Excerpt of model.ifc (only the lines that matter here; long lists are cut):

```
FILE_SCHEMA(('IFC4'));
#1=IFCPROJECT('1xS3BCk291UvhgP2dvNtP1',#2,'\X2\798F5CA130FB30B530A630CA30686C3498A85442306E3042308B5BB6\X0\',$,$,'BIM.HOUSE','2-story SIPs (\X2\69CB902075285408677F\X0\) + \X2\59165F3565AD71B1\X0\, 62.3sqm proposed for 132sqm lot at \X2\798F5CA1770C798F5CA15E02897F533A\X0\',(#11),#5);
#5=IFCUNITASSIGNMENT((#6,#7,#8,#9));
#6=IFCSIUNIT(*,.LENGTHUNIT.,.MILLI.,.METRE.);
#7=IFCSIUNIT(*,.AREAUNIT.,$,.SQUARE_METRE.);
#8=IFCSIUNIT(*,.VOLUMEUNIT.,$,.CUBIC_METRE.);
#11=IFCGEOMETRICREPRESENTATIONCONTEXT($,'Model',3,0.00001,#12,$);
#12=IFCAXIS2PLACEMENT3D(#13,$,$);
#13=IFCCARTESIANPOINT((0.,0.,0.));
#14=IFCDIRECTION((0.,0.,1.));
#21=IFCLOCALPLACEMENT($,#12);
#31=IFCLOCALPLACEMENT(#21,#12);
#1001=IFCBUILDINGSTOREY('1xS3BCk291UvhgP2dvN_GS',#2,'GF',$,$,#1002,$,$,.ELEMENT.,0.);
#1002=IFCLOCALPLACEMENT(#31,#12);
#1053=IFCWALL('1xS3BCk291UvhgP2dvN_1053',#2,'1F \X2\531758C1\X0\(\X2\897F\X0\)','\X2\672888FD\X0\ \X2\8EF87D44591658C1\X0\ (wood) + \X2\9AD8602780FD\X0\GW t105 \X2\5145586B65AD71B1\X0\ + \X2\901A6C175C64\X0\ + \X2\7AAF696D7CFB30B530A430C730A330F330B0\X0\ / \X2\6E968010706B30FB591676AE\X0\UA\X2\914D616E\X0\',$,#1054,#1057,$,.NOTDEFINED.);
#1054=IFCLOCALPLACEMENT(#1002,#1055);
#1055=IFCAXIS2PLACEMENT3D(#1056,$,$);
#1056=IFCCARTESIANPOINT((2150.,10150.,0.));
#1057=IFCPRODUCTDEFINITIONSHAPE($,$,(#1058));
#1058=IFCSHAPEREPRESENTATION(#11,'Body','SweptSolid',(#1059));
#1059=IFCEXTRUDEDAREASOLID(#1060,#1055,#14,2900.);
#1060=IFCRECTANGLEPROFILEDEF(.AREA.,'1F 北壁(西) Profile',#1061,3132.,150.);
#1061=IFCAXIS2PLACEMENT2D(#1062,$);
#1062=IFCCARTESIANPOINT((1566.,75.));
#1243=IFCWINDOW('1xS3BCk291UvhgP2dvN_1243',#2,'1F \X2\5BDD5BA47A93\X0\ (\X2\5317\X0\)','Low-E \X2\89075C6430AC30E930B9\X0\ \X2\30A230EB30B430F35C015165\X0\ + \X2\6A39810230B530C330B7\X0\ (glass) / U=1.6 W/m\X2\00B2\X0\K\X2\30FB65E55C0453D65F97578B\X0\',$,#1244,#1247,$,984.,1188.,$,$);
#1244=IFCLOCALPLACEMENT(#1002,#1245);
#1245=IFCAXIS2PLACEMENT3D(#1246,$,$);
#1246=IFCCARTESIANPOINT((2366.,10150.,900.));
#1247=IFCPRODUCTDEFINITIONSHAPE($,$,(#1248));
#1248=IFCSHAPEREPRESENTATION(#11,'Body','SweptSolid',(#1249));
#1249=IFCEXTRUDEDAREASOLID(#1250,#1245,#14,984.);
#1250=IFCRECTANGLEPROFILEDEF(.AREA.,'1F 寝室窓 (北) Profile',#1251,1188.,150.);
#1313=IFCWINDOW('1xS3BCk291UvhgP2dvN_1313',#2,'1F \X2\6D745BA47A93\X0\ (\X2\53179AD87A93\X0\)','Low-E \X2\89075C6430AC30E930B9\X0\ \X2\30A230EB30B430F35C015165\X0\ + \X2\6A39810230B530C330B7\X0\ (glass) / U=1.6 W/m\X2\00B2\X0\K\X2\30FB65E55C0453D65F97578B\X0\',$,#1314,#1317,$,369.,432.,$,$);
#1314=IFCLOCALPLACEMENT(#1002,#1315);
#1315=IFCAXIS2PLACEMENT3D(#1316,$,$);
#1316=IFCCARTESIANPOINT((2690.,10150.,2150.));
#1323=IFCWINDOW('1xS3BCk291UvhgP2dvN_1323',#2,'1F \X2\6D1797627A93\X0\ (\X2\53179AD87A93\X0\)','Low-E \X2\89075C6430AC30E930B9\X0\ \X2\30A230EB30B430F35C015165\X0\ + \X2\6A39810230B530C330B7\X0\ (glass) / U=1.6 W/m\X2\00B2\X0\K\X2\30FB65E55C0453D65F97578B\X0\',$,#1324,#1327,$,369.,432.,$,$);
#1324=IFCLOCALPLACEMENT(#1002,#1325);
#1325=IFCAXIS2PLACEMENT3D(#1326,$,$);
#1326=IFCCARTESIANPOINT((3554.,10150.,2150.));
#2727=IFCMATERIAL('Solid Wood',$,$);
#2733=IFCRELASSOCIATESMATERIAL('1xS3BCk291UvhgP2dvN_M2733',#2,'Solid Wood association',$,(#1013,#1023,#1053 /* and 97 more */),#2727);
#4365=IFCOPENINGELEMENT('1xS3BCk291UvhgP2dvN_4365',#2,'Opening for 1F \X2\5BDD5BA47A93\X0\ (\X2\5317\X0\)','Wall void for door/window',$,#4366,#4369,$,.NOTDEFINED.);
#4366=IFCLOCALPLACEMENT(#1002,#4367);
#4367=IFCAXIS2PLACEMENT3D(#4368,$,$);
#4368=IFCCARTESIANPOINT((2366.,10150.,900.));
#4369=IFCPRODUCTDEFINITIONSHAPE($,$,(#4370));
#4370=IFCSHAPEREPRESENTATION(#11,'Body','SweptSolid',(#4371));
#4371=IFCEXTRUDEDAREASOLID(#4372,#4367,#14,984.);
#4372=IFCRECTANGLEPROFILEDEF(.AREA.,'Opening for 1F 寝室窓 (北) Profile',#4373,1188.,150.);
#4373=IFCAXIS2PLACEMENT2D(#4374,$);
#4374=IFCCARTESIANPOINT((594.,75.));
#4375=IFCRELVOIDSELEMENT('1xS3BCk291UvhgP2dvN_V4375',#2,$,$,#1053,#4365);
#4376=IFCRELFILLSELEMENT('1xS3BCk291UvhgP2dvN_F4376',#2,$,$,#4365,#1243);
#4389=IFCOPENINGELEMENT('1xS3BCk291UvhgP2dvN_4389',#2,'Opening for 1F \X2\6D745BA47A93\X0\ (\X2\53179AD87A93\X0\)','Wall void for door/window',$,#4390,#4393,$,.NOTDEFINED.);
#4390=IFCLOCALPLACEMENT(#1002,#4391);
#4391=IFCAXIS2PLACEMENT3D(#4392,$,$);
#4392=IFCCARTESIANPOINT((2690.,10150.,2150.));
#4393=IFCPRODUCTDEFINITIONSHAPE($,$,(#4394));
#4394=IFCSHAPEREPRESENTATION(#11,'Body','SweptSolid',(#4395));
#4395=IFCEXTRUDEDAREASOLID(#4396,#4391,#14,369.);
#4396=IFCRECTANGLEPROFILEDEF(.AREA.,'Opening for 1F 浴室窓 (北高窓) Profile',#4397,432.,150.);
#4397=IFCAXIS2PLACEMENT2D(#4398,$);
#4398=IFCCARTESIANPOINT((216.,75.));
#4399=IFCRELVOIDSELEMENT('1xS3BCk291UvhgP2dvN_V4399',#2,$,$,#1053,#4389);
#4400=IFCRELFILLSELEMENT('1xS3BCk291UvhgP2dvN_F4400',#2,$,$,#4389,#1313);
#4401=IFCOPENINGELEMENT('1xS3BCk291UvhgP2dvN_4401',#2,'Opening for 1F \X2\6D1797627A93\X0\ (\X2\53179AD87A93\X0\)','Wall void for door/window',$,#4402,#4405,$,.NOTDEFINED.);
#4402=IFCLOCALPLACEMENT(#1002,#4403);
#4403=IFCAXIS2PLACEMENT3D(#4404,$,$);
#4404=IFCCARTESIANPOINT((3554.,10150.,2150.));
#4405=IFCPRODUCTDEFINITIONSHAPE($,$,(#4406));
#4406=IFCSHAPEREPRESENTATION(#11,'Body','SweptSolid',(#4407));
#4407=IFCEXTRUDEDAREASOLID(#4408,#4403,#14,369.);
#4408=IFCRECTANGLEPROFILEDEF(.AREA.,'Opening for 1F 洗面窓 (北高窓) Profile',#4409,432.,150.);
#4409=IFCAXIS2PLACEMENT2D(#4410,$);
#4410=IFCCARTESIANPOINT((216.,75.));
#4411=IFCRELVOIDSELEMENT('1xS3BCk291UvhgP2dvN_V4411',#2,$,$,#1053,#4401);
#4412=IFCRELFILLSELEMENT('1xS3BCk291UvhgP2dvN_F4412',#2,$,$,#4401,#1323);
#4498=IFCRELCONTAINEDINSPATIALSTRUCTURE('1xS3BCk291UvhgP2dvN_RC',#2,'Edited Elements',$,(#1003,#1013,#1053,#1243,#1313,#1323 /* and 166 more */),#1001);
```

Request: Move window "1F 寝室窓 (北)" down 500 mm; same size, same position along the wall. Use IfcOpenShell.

```python
import numpy as np
import ifcopenshell
import ifcopenshell.api.geometry
import ifcopenshell.util.placement
import ifcopenshell.util.unit

model = ifcopenshell.open("model.ifc")
unit_scale = ifcopenshell.util.unit.calculate_unit_scale(model)

window = model.by_guid("1xS3BCk291UvhgP2dvN_1243")
opening = window.FillsVoids[0].RelatingOpeningElement
dz = -500.0

shift = np.array([0.0, 0.0, dz])
# The window is not placed relative to its opening, so move both.
for product in (opening, window):
    matrix = ifcopenshell.util.placement.get_local_placement(product.ObjectPlacement)
    matrix[:3, 3] += shift
    ifcopenshell.api.geometry.edit_object_placement(model, product=product, matrix=matrix, is_si=False)

print(f"moved by {dz * unit_scale:+.3f} m")

model.write("model_rev.ifc")
```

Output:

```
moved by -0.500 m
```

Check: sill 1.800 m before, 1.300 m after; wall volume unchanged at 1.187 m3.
